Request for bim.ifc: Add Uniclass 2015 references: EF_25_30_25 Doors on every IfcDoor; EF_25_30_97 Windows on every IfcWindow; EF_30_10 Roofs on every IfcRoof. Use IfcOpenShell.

First a look at what the model holds.

```python
import ifcopenshell

model = ifcopenshell.open("bim.ifc")
print(model.schema)
print("classifications:", [c.Name for c in model.by_type("IfcClassification")])
for ifc_class in ("IfcDoor", "IfcRoof", "IfcStair", "IfcWall", "IfcWindow"):
    print(ifc_class, len(model.by_type(ifc_class)))
```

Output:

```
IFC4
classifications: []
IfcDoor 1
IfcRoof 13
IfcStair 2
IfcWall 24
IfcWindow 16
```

```python
import ifcopenshell
import ifcopenshell.api.classification

model = ifcopenshell.open("bim.ifc")

system = ifcopenshell.api.classification.add_classification(model, classification="Uniclass 2015")

codes = {
    "IfcDoor": ("EF_25_30_25", "Doors"),
    "IfcWindow": ("EF_25_30_97", "Windows"),
    "IfcRoof": ("EF_30_10", "Roofs"),
}
for ifc_class, (code, name) in codes.items():
    products = model.by_type(ifc_class)
    ifcopenshell.api.classification.add_reference(
        model, products=products, classification=system, identification=code, name=name
    )
    print(code, len(products))

model.write("bim_rev.ifc")
```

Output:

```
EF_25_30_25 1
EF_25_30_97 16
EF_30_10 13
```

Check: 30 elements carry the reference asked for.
